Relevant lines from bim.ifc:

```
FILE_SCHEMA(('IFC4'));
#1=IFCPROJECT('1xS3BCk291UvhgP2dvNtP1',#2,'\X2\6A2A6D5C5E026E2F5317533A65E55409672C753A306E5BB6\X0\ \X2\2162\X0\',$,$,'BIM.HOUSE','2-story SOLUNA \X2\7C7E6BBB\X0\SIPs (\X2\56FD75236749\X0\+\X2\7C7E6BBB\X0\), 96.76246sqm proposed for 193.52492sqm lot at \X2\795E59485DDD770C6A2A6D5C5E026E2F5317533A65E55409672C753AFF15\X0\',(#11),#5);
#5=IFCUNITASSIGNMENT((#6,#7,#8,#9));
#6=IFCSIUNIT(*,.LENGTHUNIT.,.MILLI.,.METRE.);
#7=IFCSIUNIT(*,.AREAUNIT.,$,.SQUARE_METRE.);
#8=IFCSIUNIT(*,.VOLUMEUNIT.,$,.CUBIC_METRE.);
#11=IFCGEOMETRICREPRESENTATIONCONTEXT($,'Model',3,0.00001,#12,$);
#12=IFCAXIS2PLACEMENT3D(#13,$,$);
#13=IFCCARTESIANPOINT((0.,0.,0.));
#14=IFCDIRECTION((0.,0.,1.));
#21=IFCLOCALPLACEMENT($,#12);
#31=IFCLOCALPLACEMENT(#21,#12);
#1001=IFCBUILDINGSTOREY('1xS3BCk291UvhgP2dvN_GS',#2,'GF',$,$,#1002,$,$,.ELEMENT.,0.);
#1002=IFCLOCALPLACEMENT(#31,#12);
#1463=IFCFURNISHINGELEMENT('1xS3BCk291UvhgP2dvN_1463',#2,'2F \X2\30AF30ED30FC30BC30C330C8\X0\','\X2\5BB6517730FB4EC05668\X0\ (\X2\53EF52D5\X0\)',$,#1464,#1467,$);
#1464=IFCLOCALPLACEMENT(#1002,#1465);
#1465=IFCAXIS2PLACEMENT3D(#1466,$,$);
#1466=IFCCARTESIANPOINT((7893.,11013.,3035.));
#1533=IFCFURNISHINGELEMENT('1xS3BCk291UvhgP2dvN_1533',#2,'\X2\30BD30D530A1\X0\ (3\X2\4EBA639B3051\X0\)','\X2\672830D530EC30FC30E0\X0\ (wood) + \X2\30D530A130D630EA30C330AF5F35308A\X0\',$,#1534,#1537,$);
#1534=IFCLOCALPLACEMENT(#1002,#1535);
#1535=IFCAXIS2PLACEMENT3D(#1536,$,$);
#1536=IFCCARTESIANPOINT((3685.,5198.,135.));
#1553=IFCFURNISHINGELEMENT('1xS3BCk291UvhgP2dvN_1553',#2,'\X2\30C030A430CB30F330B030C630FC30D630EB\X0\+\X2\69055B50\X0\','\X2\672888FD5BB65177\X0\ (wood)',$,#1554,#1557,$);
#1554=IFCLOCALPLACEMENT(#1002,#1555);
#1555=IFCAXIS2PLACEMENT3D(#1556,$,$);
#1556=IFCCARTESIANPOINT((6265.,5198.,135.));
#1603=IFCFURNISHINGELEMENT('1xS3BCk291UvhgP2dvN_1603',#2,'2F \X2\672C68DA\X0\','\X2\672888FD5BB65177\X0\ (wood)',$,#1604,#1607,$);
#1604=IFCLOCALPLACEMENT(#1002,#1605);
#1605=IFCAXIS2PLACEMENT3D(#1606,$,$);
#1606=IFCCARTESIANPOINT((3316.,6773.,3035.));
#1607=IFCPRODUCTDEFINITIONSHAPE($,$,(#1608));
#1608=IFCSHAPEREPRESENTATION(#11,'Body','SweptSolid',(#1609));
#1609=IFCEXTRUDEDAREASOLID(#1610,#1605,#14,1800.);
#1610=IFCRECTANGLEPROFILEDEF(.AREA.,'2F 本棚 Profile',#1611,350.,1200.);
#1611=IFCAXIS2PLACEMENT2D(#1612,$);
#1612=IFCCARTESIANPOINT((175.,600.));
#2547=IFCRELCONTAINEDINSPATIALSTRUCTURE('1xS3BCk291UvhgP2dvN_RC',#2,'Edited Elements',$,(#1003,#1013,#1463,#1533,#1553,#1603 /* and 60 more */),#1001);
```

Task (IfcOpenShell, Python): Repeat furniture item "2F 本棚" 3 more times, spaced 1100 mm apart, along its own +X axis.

```python
import ifcopenshell
import ifcopenshell.api.geometry
import ifcopenshell.api.root
import ifcopenshell.util.element
import ifcopenshell.util.placement

model = ifcopenshell.open("bim.ifc")


def reuse_history(source, copy):
    """copy_class also copies each property set's owner history, people and application; keep the originals."""
    for rel in copy.IsDefinedBy:
        if rel.is_a("IfcRelDefinesByProperties") and (history := rel.RelatingPropertyDefinition.OwnerHistory):
            rel.RelatingPropertyDefinition.OwnerHistory = source.OwnerHistory
            ifcopenshell.util.element.remove_deep2(model, history)


source = model.by_guid("1xS3BCk291UvhgP2dvN_1603")
base = ifcopenshell.util.placement.get_local_placement(source.ObjectPlacement)
step = base[:3, 0] * 1100.0

for i in range(1, 4):
    copy = ifcopenshell.api.root.copy_class(model, product=source)
    copy.Representation = ifcopenshell.util.element.copy_deep(
        model, source.Representation, exclude=["IfcGeometricRepresentationContext", "IfcRepresentationMap"]
    )
    reuse_history(source, copy)
    matrix = base.copy()
    matrix[:3, 3] += i * step
    print("added at", matrix[:3, 3].round(3) + 0.0)
    ifcopenshell.api.geometry.edit_object_placement(model, product=copy, matrix=matrix, is_si=False)

model.write("bim-out.ifc")
```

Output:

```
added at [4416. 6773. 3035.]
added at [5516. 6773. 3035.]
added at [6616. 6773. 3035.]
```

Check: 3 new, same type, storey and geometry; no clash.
